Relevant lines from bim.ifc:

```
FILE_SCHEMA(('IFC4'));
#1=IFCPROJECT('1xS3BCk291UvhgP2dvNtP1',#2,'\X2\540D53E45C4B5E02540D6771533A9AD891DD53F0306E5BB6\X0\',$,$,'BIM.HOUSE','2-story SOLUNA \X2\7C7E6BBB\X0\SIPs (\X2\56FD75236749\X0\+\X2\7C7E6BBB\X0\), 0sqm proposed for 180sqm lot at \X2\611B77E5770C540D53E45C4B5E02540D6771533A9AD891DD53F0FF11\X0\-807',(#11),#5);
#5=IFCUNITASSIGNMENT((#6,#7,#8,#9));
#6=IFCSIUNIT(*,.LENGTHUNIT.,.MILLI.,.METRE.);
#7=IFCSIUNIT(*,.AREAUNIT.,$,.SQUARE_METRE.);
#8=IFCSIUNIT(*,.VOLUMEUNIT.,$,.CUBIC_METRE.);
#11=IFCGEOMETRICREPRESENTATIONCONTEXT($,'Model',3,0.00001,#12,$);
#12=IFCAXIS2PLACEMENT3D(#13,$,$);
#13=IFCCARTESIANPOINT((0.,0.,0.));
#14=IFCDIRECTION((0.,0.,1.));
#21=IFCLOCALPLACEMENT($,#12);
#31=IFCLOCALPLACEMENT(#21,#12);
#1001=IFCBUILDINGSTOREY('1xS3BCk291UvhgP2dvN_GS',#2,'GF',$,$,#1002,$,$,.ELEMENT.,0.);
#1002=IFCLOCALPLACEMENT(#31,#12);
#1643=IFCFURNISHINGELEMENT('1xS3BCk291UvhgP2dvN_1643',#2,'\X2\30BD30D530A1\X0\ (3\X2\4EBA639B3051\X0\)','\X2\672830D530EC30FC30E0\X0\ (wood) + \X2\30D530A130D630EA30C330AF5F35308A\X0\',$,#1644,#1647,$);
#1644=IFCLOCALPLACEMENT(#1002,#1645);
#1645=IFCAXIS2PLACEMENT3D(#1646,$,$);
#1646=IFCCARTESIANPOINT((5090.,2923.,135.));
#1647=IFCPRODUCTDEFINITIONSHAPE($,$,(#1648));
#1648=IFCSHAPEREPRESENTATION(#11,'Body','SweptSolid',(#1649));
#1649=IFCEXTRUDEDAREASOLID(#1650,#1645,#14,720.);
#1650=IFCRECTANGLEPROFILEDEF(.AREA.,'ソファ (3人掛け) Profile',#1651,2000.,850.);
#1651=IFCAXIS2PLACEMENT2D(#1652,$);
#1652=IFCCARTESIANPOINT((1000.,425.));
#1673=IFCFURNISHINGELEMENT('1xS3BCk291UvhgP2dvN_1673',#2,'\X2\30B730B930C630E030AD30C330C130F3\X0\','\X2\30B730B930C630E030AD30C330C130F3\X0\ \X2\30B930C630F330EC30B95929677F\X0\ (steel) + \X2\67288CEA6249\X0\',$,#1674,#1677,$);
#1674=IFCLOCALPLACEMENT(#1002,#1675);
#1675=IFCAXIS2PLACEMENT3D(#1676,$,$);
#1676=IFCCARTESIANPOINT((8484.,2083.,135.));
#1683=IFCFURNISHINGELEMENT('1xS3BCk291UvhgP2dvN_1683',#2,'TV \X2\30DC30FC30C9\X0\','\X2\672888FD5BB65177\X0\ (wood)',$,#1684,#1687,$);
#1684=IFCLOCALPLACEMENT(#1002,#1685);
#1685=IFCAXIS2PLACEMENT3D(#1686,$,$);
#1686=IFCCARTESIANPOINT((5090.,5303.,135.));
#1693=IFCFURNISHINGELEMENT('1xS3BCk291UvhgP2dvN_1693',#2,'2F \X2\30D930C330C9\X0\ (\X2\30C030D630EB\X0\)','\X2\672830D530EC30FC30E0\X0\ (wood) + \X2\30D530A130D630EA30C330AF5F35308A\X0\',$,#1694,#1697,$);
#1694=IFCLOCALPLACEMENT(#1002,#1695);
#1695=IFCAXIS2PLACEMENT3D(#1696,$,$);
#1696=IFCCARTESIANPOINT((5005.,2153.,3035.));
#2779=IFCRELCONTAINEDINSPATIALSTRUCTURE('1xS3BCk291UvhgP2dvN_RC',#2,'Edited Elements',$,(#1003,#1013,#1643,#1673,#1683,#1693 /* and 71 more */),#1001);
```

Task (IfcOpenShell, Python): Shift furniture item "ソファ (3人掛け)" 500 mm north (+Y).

```python
import ifcopenshell
import ifcopenshell.api.geometry
import ifcopenshell.util.placement

model = ifcopenshell.open("bim.ifc")

item = model.by_id(1643)
matrix = ifcopenshell.util.placement.get_local_placement(item.ObjectPlacement)
matrix[1, 3] += 500.0
ifcopenshell.api.geometry.edit_object_placement(model, product=item, matrix=matrix, is_si=False)

print(ifcopenshell.util.placement.get_local_placement(item.ObjectPlacement).round(3) + 0.0)

model.write("bim_rev.ifc")
```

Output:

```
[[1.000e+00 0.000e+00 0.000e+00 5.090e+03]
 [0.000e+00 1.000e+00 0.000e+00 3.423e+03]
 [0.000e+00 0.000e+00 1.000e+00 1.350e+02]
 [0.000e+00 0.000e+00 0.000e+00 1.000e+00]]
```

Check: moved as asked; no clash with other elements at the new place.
